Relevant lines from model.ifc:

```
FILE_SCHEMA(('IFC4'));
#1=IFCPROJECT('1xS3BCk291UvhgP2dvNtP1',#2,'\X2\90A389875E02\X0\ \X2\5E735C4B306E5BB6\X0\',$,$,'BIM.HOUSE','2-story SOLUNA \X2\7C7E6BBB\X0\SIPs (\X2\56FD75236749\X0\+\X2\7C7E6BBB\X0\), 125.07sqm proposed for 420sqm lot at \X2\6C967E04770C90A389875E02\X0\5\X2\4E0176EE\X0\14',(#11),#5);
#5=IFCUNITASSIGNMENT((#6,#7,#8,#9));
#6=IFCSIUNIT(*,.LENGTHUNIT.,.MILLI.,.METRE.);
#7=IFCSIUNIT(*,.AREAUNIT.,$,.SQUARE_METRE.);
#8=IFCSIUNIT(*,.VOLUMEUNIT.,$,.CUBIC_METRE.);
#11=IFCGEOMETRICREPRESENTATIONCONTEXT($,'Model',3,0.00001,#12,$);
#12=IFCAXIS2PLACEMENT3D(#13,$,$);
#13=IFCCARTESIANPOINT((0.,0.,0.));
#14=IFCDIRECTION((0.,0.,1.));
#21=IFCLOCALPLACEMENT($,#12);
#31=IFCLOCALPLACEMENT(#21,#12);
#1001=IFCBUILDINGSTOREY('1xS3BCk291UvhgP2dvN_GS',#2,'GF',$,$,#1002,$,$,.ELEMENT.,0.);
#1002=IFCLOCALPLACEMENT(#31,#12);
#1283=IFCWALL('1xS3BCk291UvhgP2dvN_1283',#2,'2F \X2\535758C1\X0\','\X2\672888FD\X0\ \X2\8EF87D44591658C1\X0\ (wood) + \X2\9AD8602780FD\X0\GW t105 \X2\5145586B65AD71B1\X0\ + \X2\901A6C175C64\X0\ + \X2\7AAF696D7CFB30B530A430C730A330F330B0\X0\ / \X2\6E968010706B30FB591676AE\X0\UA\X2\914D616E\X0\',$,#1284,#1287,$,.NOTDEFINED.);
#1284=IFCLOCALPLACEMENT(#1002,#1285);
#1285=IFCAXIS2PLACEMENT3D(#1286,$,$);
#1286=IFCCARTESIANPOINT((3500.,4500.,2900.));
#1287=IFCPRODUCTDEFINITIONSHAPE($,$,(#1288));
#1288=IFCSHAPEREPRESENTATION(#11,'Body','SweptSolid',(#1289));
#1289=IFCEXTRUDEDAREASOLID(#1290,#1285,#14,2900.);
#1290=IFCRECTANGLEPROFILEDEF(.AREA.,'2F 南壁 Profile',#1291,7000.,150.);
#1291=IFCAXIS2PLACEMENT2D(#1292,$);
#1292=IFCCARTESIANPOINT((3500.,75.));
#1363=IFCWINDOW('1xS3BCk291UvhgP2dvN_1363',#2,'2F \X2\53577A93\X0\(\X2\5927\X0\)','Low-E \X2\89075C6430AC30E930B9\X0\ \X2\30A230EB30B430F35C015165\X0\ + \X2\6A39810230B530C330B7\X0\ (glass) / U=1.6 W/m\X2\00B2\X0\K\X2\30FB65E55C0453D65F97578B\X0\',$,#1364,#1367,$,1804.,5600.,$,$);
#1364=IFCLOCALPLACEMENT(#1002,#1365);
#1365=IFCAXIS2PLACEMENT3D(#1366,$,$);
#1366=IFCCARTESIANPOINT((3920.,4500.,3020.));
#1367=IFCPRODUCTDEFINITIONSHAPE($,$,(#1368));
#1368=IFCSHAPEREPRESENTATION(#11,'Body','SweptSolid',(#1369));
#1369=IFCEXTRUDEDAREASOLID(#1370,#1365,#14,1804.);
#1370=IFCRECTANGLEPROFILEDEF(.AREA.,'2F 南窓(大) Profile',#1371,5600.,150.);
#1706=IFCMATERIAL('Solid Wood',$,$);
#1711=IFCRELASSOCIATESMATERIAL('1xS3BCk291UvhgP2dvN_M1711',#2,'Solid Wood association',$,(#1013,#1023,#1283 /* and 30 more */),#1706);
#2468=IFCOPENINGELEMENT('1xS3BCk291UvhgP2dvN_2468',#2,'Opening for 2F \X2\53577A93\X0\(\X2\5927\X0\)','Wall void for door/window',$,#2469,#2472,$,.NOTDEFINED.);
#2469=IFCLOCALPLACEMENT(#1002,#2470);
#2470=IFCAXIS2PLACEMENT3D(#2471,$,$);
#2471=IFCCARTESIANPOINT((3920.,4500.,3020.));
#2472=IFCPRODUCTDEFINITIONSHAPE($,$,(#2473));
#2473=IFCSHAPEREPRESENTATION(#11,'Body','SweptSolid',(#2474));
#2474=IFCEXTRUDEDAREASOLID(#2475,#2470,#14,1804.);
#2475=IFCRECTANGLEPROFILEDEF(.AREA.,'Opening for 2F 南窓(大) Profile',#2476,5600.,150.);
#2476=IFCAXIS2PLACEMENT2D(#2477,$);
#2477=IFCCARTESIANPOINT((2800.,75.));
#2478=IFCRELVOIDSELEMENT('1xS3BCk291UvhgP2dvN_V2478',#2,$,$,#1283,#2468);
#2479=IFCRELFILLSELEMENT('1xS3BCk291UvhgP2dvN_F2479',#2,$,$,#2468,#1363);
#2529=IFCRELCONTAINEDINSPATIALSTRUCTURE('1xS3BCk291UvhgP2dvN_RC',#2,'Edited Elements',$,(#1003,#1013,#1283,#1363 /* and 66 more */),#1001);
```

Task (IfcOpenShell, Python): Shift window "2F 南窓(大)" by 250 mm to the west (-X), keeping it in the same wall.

```python
import ifcopenshell
import ifcopenshell.api.geometry
import ifcopenshell.util.placement

model = ifcopenshell.open("model.ifc")

window = model.by_guid("1xS3BCk291UvhgP2dvN_1363")
opening = window.FillsVoids[0].RelatingOpeningElement
wall = opening.VoidsElements[0].RelatingBuildingElement

wall_matrix = ifcopenshell.util.placement.get_local_placement(wall.ObjectPlacement)
shift = wall_matrix[:3, 0] * -250.0
before = ifcopenshell.util.placement.get_local_placement(window.ObjectPlacement)[:3, 3].copy()

# The window is not placed relative to its opening, so move both.
for product in (opening, window):
    matrix = ifcopenshell.util.placement.get_local_placement(product.ObjectPlacement)
    matrix[:3, 3] += shift
    ifcopenshell.api.geometry.edit_object_placement(model, product=product, matrix=matrix, is_si=False)

after = ifcopenshell.util.placement.get_local_placement(window.ObjectPlacement)[:3, 3]
print("window moved by", (after - before).round(3) + 0.0)

model.write("model-out.ifc")
```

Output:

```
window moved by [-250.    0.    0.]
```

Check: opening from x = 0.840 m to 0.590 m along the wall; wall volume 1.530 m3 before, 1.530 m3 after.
